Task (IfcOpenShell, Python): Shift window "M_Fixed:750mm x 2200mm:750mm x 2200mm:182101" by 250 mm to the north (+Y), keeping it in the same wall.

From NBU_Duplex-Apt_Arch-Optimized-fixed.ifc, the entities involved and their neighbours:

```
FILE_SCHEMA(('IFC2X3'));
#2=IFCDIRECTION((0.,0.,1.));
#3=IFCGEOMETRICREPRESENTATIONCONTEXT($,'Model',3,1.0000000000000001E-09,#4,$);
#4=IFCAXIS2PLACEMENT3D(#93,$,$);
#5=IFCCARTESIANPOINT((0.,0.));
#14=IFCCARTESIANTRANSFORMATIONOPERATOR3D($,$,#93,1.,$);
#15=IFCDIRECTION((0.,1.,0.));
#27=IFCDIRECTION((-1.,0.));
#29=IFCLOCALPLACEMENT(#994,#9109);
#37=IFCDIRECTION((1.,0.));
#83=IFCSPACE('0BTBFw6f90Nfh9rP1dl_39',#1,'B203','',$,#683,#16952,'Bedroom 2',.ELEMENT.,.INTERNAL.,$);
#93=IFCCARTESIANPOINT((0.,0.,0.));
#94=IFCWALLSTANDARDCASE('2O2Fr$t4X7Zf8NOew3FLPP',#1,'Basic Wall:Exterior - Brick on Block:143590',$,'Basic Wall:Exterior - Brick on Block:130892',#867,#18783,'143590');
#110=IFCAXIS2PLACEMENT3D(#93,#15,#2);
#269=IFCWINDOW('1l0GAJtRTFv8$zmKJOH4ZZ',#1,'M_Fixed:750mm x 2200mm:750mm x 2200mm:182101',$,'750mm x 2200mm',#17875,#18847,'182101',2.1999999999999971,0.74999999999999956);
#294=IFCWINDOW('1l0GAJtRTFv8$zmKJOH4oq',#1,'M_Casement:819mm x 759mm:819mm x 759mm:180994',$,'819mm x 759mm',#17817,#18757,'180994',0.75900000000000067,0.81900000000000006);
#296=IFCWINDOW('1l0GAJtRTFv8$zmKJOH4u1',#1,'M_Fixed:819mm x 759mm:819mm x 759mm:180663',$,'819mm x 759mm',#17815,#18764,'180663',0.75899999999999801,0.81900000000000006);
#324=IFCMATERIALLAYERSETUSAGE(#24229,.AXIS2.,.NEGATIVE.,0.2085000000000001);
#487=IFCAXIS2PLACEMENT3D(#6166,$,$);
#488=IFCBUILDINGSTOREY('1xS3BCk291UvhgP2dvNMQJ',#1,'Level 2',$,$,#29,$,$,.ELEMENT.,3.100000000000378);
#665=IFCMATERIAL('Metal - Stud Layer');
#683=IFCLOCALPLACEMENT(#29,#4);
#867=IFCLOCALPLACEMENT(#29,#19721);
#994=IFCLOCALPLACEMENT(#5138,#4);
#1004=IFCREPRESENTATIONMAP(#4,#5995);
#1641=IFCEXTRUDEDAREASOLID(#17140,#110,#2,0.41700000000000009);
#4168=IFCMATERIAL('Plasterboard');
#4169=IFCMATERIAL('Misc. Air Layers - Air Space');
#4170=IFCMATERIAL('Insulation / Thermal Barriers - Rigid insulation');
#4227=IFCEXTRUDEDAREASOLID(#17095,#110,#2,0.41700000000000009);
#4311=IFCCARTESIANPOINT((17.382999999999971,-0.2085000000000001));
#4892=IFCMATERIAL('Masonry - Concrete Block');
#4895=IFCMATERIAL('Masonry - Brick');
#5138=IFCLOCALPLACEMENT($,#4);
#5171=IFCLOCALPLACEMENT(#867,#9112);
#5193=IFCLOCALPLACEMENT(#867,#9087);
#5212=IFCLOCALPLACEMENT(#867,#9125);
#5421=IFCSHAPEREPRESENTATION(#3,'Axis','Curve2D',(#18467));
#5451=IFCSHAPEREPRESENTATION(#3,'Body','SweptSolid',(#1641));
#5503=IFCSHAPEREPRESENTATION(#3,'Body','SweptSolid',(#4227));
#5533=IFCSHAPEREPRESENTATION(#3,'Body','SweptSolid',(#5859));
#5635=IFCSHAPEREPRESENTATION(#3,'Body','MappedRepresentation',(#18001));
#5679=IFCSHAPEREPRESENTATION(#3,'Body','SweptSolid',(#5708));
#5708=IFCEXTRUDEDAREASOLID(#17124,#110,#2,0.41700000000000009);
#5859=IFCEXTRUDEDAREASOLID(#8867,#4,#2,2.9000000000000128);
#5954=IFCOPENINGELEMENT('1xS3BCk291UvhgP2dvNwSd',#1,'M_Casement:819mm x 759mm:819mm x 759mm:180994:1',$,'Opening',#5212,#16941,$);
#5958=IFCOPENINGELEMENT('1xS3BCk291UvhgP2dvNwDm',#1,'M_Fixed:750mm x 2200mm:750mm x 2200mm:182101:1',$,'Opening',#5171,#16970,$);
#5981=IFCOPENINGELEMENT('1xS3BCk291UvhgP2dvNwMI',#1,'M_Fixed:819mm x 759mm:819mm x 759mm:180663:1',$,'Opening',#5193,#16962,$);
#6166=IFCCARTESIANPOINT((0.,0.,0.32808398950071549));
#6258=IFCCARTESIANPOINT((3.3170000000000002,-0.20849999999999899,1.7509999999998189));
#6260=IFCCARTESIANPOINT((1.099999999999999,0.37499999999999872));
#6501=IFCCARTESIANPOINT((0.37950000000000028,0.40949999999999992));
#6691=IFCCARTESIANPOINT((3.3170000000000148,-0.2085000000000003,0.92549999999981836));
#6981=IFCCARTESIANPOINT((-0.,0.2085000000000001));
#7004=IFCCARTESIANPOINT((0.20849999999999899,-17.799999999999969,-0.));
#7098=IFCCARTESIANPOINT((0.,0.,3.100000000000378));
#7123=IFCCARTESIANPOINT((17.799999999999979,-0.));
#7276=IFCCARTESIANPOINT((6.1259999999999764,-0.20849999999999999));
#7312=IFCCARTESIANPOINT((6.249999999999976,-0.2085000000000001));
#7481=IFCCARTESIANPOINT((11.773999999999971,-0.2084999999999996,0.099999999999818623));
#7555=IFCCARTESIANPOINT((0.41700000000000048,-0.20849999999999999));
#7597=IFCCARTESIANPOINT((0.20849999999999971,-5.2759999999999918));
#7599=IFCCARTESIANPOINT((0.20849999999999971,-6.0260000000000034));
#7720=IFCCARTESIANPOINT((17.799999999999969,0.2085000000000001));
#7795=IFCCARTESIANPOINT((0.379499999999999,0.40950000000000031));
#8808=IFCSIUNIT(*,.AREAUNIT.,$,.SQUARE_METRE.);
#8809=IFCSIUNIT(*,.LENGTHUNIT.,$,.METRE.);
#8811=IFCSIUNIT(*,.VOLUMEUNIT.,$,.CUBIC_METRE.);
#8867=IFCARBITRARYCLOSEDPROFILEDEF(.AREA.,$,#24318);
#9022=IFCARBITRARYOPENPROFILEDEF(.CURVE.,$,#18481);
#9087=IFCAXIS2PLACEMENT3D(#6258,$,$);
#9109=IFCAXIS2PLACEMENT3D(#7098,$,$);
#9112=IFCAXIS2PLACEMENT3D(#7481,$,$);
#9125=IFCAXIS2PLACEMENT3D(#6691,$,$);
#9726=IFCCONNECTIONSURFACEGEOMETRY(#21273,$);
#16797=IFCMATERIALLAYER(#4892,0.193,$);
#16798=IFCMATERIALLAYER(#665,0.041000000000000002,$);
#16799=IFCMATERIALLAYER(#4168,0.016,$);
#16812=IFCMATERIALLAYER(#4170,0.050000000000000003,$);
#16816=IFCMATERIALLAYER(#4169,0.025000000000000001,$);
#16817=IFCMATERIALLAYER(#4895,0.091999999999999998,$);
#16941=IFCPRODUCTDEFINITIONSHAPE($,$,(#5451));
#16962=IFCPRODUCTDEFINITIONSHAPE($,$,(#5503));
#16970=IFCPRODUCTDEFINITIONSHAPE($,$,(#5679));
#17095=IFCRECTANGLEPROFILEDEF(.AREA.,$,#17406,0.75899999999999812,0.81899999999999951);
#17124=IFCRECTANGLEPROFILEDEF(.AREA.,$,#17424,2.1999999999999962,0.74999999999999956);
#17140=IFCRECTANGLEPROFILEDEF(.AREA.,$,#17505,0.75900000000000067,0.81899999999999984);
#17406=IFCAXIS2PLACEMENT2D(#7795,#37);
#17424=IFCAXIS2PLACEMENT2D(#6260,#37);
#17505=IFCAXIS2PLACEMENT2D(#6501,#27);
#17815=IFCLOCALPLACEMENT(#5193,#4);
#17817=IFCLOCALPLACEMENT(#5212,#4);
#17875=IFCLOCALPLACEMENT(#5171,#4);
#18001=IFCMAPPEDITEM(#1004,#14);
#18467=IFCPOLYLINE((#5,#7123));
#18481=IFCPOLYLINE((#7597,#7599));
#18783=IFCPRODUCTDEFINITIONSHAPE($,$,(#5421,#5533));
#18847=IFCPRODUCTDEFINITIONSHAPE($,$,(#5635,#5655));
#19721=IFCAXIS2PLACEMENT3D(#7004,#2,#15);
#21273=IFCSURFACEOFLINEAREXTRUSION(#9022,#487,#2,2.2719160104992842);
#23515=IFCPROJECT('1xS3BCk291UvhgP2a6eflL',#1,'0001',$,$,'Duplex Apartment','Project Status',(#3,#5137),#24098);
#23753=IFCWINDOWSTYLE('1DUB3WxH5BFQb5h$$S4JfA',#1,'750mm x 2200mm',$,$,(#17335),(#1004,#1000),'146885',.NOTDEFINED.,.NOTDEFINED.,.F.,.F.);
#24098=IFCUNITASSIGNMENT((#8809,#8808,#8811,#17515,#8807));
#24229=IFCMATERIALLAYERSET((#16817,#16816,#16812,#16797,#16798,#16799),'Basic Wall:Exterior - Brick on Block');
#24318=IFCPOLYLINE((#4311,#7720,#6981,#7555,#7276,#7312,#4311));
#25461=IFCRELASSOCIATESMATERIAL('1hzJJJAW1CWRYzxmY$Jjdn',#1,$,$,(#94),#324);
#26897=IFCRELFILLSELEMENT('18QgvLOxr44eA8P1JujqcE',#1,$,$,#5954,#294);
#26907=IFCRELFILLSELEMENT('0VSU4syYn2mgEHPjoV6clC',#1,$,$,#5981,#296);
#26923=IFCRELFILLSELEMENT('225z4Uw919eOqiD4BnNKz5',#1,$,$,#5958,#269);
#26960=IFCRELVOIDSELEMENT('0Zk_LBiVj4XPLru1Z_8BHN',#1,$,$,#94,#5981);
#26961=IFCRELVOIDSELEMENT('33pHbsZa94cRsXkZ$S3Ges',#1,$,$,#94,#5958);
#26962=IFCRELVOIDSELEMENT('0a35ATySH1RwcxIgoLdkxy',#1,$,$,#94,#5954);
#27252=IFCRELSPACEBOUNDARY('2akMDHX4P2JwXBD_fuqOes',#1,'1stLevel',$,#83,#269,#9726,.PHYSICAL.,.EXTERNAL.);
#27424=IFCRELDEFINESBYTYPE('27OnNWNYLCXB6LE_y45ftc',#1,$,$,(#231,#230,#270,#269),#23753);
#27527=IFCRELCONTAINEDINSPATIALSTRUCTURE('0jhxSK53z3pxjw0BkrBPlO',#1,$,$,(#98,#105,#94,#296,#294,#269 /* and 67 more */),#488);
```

```python
import numpy as np
import ifcopenshell
import ifcopenshell.api.geometry
import ifcopenshell.util.placement
import ifcopenshell.util.unit

model = ifcopenshell.open("NBU_Duplex-Apt_Arch-Optimized-fixed.ifc")
unit_scale = ifcopenshell.util.unit.calculate_unit_scale(model)

window = model.by_guid("1l0GAJtRTFv8$zmKJOH4ZZ")
opening = window.FillsVoids[0].RelatingOpeningElement
wall = opening.VoidsElements[0].RelatingBuildingElement

wall_matrix = ifcopenshell.util.placement.get_local_placement(wall.ObjectPlacement)
shift = wall_matrix[:3, 0] * 0.25 / unit_scale
before = ifcopenshell.util.placement.get_local_placement(window.ObjectPlacement)[:3, 3].copy()

# The window is placed relative to its opening, so it follows when the opening moves.
matrix = ifcopenshell.util.placement.get_local_placement(opening.ObjectPlacement)
matrix[:3, 3] += shift
ifcopenshell.api.geometry.edit_object_placement(
    model, product=opening, matrix=matrix, is_si=False, should_transform_children=True
)

# Space boundary surfaces are stored in each space's coordinates; move them too.
for rel in window.ProvidesBoundaries:
    if not rel.ConnectionGeometry:
        continue
    surface = rel.ConnectionGeometry.SurfaceOnRelatingElement
    space_matrix = ifcopenshell.util.placement.get_local_placement(rel.RelatingSpace.ObjectPlacement)
    point = np.array(surface.Position.Location.Coordinates) + space_matrix[:3, :3].T @ shift
    surface.Position = model.createIfcAxis2Placement3D(
        model.createIfcCartesianPoint(point.tolist()), surface.Position.Axis, surface.Position.RefDirection
    )

after = ifcopenshell.util.placement.get_local_placement(window.ObjectPlacement)[:3, 3]
print("window moved by", (after - before).round(3) + 0.0)

model.write("NBU_Duplex-Apt_Arch-Optimized-fixed_v2.ifc")
```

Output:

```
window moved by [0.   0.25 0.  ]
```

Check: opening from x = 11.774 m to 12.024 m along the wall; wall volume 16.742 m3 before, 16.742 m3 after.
